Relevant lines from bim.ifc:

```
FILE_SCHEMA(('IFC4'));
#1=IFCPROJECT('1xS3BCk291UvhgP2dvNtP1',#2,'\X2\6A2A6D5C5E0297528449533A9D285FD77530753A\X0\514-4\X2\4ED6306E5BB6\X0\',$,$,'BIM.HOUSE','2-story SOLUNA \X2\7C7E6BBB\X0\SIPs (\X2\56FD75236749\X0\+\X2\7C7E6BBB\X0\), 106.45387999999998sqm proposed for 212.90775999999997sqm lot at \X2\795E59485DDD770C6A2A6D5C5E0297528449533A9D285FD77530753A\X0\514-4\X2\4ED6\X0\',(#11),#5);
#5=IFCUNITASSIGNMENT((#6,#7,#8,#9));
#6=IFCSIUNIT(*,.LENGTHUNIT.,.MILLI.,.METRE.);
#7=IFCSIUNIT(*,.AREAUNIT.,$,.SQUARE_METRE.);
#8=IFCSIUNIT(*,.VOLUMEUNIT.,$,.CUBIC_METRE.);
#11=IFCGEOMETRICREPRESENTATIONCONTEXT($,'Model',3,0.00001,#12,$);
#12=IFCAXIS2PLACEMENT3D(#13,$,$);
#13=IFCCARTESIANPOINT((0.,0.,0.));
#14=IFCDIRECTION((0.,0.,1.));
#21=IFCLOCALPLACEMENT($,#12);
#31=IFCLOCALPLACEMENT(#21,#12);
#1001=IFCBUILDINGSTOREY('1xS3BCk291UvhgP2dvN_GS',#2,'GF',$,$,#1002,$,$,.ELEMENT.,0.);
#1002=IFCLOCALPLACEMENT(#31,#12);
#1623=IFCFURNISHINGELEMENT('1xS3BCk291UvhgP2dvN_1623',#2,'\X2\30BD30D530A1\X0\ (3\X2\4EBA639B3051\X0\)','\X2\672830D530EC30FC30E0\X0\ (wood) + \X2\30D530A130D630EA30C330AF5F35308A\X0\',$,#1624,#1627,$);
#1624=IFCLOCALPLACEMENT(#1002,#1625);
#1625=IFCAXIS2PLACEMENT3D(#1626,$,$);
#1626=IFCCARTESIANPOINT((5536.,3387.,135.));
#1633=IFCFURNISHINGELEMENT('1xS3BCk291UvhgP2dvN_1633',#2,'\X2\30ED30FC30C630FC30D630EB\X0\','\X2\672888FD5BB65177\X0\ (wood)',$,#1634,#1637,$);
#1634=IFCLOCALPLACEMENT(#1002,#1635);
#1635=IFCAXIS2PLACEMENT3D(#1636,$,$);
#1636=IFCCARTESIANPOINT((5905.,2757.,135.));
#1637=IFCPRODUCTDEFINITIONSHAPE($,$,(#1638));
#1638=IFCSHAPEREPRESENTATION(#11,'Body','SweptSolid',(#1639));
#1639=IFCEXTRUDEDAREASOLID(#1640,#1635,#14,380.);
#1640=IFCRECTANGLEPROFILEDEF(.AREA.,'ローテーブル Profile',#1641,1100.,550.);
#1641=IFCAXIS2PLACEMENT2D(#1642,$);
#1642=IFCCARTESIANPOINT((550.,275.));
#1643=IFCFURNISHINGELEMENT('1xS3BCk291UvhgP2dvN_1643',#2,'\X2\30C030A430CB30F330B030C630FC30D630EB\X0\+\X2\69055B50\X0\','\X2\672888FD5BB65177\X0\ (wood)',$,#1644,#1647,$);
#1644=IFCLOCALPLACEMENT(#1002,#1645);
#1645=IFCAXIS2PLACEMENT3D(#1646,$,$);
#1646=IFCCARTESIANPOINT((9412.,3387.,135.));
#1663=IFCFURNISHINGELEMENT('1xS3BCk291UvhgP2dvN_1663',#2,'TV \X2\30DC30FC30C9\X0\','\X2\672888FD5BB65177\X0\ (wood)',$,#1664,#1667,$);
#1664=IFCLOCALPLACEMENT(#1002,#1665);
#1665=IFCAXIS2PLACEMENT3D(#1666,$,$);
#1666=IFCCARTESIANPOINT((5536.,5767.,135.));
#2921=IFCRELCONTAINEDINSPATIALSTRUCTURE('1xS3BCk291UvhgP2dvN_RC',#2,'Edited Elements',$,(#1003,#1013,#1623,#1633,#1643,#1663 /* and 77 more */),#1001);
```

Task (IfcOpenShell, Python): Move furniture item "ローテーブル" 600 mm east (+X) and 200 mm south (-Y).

```python
import ifcopenshell
import ifcopenshell.api.geometry
import ifcopenshell.util.placement

model = ifcopenshell.open("bim.ifc")

item = model.by_guid("1xS3BCk291UvhgP2dvN_1633")
matrix = ifcopenshell.util.placement.get_local_placement(item.ObjectPlacement)
matrix[0, 3] += 600.0
matrix[1, 3] -= 200.0
ifcopenshell.api.geometry.edit_object_placement(model, product=item, matrix=matrix, is_si=False)

print(ifcopenshell.util.placement.get_local_placement(item.ObjectPlacement).round(3) + 0.0)

model.write("bim_updated.ifc")
```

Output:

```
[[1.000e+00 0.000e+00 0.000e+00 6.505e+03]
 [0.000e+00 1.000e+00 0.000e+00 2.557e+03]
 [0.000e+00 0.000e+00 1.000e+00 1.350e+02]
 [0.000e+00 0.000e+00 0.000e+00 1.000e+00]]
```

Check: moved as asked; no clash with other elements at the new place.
